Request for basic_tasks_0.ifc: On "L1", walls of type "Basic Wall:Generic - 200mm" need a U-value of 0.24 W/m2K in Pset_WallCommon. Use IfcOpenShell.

First a look at what the model holds.

```python
import ifcopenshell
import ifcopenshell.util.element

model = ifcopenshell.open("basic_tasks_0.ifc")
print(model.schema)
storey = next(s for s in model.by_type("IfcBuildingStorey") if s.Name == "L1")
walls = [e for e in ifcopenshell.util.element.get_decomposition(storey) if e.is_a("IfcWall")]
seen = {}
for e in walls:
    element_type = ifcopenshell.util.element.get_type(e)
    key = (element_type.Name if element_type != e and element_type else None, ifcopenshell.util.element.get_pset(e, "Pset_WallCommon", "ThermalTransmittance"))
    seen[key] = seen.get(key, 0) + 1
for (name, value), count in sorted(seen.items(), key=str):
    print(count, "x", name, "|", value)
```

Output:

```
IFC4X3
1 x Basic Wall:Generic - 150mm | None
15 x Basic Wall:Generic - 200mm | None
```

```python
import ifcopenshell
import ifcopenshell.api.pset
import ifcopenshell.util.element

model = ifcopenshell.open("basic_tasks_0.ifc")

storey = next(s for s in model.by_type("IfcBuildingStorey") if s.Name == "L1")
walls = [e for e in ifcopenshell.util.element.get_decomposition(storey) if e.is_a("IfcWall")]

count = 0
for e in walls:
    element_type = ifcopenshell.util.element.get_type(e)
    if element_type in (None, e) or element_type.Name != "Basic Wall:Generic - 200mm":
        continue
    # add_pset returns the element's existing set when there is one.
    pset = ifcopenshell.api.pset.add_pset(model, product=e, name="Pset_WallCommon")
    ifcopenshell.api.pset.edit_pset(model, pset=pset, properties={"ThermalTransmittance": 0.24})
    count += 1

print(count, "walls updated")

model.write("basic_tasks_0-out.ifc")
```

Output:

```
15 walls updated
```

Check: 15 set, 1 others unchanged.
